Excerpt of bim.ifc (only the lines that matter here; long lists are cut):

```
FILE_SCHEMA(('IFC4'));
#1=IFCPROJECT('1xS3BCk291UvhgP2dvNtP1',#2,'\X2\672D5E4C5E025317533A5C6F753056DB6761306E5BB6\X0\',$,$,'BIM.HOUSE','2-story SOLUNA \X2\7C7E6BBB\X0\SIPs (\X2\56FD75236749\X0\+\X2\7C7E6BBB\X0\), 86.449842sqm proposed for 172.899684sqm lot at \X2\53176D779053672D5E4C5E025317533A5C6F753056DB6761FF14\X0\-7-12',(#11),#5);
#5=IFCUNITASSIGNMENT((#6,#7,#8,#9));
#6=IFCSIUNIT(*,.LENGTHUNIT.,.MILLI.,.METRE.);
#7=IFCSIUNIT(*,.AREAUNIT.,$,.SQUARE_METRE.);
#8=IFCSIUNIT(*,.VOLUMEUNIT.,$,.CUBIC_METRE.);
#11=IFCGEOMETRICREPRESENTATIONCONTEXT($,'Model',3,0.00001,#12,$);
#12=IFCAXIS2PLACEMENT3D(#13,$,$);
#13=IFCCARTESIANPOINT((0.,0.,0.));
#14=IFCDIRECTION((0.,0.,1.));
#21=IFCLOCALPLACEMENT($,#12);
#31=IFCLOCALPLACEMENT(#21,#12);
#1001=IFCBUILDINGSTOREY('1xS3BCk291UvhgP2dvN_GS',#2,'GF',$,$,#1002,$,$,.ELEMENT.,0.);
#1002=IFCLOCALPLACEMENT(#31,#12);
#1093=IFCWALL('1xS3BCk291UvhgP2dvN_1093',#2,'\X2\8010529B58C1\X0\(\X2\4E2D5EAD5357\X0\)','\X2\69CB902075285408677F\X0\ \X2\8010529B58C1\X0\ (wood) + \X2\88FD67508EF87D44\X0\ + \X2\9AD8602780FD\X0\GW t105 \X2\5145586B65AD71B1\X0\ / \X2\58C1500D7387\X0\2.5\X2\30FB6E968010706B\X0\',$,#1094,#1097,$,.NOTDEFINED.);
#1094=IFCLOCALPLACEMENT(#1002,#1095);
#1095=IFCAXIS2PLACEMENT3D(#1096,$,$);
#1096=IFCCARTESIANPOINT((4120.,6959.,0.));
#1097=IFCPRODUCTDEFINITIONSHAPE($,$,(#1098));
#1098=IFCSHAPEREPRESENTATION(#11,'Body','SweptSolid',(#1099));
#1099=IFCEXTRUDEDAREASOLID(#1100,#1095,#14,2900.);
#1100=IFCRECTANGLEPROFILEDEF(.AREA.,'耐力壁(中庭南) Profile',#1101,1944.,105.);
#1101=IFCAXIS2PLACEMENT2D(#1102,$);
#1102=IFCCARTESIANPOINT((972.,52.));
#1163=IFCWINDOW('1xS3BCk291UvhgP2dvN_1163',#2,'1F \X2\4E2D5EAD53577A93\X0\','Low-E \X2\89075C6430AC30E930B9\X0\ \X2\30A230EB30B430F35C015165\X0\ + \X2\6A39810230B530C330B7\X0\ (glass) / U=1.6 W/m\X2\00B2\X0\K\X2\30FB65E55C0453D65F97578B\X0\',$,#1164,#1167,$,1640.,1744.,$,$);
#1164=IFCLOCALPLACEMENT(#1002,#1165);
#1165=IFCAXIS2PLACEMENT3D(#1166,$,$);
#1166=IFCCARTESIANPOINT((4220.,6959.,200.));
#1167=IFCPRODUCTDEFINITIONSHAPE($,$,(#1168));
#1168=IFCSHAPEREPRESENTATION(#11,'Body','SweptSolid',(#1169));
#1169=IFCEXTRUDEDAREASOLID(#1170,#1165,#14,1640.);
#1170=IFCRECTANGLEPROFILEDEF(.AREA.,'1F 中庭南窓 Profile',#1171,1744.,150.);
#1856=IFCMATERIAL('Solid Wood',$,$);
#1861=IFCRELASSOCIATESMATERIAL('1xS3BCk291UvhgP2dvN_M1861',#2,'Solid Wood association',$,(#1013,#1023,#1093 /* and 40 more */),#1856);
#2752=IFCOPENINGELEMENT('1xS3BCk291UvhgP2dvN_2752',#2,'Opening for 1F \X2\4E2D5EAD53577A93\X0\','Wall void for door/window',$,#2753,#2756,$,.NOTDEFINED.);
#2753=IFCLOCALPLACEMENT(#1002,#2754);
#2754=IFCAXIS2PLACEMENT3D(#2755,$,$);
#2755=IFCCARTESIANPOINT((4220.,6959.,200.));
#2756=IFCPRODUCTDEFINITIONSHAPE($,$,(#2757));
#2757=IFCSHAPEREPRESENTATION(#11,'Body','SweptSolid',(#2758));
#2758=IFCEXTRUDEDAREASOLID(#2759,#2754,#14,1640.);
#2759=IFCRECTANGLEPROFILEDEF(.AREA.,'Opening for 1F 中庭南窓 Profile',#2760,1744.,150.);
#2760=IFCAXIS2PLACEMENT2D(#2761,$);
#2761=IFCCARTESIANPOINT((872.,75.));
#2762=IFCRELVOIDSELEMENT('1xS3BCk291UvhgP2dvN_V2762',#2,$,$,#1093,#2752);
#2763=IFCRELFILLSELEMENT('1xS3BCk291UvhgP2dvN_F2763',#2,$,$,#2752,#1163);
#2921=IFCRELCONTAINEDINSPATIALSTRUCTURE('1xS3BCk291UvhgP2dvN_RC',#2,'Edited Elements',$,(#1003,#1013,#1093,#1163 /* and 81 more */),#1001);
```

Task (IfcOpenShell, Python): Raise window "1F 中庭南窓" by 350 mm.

```python
import numpy as np
import ifcopenshell
import ifcopenshell.api.geometry
import ifcopenshell.util.placement
import ifcopenshell.util.unit

model = ifcopenshell.open("bim.ifc")
unit_scale = ifcopenshell.util.unit.calculate_unit_scale(model)

window = model.by_guid("1xS3BCk291UvhgP2dvN_1163")
opening = window.FillsVoids[0].RelatingOpeningElement
dz = 350.0

shift = np.array([0.0, 0.0, dz])
# The window is not placed relative to its opening, so move both.
for product in (opening, window):
    matrix = ifcopenshell.util.placement.get_local_placement(product.ObjectPlacement)
    matrix[:3, 3] += shift
    ifcopenshell.api.geometry.edit_object_placement(model, product=product, matrix=matrix, is_si=False)

print(f"moved by {dz * unit_scale:+.3f} m")

model.write("bim_updated.ifc")
```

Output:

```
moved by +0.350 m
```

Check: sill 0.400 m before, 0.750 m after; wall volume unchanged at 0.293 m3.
